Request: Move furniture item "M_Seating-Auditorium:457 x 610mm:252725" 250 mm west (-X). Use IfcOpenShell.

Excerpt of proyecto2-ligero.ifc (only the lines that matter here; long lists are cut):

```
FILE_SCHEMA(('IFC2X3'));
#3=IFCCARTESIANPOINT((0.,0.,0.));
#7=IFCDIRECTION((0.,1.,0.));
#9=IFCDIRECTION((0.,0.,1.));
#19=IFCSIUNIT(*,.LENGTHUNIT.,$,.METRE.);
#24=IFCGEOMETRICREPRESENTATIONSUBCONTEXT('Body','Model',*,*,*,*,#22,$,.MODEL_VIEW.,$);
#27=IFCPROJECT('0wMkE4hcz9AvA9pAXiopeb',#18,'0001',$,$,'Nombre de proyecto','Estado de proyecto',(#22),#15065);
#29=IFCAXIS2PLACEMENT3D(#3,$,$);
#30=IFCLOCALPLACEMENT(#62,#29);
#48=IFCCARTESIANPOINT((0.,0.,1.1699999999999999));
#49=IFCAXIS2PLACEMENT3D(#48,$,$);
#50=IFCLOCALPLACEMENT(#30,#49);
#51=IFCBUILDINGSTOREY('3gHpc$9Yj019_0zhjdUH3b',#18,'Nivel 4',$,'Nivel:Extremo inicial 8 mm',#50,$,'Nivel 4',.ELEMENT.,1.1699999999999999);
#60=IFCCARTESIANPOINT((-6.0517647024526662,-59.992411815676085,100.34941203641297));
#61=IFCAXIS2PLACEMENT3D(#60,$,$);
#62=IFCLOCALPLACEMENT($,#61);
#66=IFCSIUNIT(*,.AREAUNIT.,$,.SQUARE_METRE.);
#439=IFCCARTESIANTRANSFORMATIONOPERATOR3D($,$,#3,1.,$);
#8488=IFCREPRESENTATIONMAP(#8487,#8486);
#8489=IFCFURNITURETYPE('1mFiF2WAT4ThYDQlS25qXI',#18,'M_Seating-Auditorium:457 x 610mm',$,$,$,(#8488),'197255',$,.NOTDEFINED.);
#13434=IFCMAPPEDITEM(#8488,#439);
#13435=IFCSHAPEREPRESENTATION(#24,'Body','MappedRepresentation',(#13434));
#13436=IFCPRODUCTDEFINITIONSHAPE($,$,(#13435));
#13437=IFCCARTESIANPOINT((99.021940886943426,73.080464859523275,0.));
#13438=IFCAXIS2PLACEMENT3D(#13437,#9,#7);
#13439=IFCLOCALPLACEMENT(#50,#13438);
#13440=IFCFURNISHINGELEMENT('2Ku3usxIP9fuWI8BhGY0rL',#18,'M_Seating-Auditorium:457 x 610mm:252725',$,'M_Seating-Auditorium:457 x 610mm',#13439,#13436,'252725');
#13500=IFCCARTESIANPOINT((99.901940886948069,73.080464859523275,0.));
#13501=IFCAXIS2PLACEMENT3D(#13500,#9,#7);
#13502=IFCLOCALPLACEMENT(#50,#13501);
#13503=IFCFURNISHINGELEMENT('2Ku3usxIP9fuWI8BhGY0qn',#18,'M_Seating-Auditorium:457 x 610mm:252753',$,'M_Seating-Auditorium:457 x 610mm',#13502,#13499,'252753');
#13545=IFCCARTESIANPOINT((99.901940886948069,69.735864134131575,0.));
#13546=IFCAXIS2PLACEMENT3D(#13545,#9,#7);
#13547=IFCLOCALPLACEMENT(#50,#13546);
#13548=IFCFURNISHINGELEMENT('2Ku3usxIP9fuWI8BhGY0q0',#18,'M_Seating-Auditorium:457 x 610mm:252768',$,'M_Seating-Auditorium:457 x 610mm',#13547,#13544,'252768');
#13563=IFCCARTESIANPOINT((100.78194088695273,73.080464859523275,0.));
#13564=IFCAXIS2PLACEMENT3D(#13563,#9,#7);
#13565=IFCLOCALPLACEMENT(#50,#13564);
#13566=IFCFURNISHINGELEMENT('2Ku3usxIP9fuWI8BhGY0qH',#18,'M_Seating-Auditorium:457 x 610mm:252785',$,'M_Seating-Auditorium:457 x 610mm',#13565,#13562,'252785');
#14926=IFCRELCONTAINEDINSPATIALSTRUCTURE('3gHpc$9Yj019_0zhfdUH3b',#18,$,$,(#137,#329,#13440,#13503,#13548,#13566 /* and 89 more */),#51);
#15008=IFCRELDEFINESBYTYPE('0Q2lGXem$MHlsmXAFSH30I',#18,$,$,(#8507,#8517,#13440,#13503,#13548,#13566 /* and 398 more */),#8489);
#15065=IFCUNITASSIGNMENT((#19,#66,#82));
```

```python
import ifcopenshell
import ifcopenshell.api.geometry
import ifcopenshell.util.placement
import ifcopenshell.util.unit

model = ifcopenshell.open("proyecto2-ligero.ifc")
unit_scale = ifcopenshell.util.unit.calculate_unit_scale(model)

item = model.by_id(13440)
matrix = ifcopenshell.util.placement.get_local_placement(item.ObjectPlacement)
matrix[0, 3] -= 0.25 / unit_scale
ifcopenshell.api.geometry.edit_object_placement(model, product=item, matrix=matrix, is_si=False)

print(ifcopenshell.util.placement.get_local_placement(item.ObjectPlacement).round(3) + 0.0)

model.write("proyecto2-ligero_edited.ifc")
```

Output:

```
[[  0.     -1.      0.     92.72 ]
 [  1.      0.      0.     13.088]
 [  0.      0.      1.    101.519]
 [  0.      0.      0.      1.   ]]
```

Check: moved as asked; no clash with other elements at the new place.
